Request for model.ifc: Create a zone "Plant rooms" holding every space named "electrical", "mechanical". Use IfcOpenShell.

First a look at what the model holds.

```python
import ifcopenshell

model = ifcopenshell.open("model.ifc")
print(model.schema)
seen = {}
for space in model.by_type("IfcSpace"):
    seen[space.LongName] = seen.get(space.LongName, 0) + 1
for name, count in sorted(seen.items(), key=str):
    print(count, "x", name)
print("zones:", [z.Name for z in model.by_type("IfcZone")][:20])
```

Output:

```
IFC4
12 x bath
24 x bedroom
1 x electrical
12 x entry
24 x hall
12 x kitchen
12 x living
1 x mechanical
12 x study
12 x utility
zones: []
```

```python
import ifcopenshell
import ifcopenshell.api.group
import ifcopenshell.api.root

model = ifcopenshell.open("model.ifc")

names = {"electrical", "mechanical"}
spaces = [s for s in model.by_type("IfcSpace") if s.LongName in names]

zone = ifcopenshell.api.root.create_entity(model, ifc_class="IfcZone", name="Plant rooms")
ifcopenshell.api.group.assign_group(model, products=spaces, group=zone)
print(len(spaces), "spaces in", zone.Name)

model.write("model_updated.ifc")
```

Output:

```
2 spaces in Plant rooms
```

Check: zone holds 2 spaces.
